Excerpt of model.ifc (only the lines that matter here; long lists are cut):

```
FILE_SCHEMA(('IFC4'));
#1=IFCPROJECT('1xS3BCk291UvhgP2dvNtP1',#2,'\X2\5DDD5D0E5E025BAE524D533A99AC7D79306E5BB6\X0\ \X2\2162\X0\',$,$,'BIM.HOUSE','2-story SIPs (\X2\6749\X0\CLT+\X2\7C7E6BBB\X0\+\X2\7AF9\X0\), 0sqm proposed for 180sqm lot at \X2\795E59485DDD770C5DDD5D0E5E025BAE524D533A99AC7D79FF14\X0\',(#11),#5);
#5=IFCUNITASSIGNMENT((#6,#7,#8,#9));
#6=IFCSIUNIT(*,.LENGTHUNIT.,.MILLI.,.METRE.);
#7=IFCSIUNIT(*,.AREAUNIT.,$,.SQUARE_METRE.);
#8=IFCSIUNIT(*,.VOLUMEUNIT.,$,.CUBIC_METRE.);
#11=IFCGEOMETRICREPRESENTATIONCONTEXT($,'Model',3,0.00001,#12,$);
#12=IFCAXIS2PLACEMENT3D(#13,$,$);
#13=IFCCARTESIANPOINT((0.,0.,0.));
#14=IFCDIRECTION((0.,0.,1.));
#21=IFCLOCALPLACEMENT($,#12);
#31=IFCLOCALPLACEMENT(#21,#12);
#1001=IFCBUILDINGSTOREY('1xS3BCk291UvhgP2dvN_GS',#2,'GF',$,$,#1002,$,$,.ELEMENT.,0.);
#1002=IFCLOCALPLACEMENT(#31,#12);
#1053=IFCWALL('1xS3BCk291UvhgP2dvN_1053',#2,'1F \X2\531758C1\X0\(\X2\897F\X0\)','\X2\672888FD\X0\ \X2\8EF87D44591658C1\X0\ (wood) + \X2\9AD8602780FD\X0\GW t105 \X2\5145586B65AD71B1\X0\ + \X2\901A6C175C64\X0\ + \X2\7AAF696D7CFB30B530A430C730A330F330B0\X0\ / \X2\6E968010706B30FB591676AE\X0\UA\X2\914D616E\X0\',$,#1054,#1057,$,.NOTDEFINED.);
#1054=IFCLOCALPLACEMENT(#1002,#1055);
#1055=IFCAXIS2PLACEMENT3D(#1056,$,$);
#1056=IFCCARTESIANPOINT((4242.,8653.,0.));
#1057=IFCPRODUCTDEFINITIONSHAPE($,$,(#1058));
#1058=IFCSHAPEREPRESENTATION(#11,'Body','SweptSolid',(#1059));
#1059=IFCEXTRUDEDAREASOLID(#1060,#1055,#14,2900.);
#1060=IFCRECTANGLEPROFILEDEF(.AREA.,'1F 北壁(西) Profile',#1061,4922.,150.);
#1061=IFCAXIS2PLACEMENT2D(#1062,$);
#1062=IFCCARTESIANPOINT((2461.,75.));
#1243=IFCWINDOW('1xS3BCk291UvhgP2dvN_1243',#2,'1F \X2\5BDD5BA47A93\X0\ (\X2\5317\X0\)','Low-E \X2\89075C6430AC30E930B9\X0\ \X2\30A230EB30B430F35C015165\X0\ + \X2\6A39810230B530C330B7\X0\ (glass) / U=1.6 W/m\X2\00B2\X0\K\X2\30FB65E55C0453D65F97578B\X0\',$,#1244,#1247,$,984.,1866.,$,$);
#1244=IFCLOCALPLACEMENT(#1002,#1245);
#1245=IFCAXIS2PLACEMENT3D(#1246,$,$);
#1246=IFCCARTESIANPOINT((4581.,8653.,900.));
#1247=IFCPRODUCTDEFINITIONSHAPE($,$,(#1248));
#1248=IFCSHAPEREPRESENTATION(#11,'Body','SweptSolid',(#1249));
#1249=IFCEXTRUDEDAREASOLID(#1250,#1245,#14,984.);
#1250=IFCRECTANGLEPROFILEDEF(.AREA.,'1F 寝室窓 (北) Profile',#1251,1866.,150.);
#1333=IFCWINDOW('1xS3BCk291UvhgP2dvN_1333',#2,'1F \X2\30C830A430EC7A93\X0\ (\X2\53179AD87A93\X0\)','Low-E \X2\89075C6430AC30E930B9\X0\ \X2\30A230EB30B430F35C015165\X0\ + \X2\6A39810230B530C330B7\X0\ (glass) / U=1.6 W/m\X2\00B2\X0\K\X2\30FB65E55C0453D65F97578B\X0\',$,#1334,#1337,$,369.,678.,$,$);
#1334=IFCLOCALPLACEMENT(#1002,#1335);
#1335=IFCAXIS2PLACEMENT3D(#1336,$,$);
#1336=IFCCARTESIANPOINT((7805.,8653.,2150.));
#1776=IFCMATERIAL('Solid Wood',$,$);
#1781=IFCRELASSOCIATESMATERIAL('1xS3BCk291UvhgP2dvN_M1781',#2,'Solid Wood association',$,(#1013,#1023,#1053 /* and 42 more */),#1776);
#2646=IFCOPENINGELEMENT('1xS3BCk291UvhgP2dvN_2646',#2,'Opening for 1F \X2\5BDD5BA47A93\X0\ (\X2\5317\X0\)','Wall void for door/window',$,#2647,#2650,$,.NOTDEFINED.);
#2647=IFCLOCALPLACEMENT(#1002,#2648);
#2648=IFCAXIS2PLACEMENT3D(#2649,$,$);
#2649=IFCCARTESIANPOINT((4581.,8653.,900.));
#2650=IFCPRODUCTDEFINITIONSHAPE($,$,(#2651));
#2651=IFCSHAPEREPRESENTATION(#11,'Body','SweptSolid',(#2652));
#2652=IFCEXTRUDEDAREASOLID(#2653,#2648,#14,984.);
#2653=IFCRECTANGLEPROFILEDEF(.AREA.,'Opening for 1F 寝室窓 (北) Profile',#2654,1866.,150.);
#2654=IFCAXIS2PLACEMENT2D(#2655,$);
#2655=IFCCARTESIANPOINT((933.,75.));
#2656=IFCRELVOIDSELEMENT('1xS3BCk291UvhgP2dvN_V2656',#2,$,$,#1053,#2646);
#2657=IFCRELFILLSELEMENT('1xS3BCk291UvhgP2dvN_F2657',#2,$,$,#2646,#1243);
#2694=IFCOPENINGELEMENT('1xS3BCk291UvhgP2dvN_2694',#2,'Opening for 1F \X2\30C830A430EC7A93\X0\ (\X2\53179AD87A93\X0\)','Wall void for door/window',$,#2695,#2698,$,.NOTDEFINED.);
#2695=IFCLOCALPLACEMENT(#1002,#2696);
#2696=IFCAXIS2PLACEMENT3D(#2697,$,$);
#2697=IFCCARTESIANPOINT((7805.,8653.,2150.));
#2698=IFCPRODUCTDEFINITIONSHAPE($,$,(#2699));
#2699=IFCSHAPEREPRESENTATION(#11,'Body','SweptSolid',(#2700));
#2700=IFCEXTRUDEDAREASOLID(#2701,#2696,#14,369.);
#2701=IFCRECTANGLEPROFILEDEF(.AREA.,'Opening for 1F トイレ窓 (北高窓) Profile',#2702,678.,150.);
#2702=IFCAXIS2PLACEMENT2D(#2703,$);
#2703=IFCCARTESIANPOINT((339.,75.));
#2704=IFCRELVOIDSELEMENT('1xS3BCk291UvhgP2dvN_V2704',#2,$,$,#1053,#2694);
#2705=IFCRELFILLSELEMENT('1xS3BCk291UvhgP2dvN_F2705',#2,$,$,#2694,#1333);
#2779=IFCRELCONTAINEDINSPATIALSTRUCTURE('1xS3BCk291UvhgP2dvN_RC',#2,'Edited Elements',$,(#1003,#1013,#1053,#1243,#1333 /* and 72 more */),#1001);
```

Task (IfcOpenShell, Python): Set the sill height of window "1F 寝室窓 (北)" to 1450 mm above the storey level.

```python
import numpy as np
import ifcopenshell
import ifcopenshell.api.geometry
import ifcopenshell.geom
import ifcopenshell.util.element
import ifcopenshell.util.placement
import ifcopenshell.util.shape
import ifcopenshell.util.unit

model = ifcopenshell.open("model.ifc")
unit_scale = ifcopenshell.util.unit.calculate_unit_scale(model)

window = model.by_guid("1xS3BCk291UvhgP2dvN_1243")
opening = window.FillsVoids[0].RelatingOpeningElement
storey = ifcopenshell.util.element.get_container(window, ifc_class="IfcBuildingStorey")
level = ifcopenshell.util.placement.get_local_placement(storey.ObjectPlacement)[2, 3]

# The opening's origin need not be at the sill, so measure its lowest point.
shape = ifcopenshell.geom.create_shape(ifcopenshell.geom.settings(), opening)
bottom = ifcopenshell.util.shape.get_shape_bottom_elevation(shape, shape.geometry) / unit_scale
dz = level + 1450.0 - bottom

shift = np.array([0.0, 0.0, dz])
# The window is not placed relative to its opening, so move both.
for product in (opening, window):
    matrix = ifcopenshell.util.placement.get_local_placement(product.ObjectPlacement)
    matrix[:3, 3] += shift
    ifcopenshell.api.geometry.edit_object_placement(model, product=product, matrix=matrix, is_si=False)

print(f"moved by {dz * unit_scale:+.3f} m")

model.write("model_updated.ifc")
```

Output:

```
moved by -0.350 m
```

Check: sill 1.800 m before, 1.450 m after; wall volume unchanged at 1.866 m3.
